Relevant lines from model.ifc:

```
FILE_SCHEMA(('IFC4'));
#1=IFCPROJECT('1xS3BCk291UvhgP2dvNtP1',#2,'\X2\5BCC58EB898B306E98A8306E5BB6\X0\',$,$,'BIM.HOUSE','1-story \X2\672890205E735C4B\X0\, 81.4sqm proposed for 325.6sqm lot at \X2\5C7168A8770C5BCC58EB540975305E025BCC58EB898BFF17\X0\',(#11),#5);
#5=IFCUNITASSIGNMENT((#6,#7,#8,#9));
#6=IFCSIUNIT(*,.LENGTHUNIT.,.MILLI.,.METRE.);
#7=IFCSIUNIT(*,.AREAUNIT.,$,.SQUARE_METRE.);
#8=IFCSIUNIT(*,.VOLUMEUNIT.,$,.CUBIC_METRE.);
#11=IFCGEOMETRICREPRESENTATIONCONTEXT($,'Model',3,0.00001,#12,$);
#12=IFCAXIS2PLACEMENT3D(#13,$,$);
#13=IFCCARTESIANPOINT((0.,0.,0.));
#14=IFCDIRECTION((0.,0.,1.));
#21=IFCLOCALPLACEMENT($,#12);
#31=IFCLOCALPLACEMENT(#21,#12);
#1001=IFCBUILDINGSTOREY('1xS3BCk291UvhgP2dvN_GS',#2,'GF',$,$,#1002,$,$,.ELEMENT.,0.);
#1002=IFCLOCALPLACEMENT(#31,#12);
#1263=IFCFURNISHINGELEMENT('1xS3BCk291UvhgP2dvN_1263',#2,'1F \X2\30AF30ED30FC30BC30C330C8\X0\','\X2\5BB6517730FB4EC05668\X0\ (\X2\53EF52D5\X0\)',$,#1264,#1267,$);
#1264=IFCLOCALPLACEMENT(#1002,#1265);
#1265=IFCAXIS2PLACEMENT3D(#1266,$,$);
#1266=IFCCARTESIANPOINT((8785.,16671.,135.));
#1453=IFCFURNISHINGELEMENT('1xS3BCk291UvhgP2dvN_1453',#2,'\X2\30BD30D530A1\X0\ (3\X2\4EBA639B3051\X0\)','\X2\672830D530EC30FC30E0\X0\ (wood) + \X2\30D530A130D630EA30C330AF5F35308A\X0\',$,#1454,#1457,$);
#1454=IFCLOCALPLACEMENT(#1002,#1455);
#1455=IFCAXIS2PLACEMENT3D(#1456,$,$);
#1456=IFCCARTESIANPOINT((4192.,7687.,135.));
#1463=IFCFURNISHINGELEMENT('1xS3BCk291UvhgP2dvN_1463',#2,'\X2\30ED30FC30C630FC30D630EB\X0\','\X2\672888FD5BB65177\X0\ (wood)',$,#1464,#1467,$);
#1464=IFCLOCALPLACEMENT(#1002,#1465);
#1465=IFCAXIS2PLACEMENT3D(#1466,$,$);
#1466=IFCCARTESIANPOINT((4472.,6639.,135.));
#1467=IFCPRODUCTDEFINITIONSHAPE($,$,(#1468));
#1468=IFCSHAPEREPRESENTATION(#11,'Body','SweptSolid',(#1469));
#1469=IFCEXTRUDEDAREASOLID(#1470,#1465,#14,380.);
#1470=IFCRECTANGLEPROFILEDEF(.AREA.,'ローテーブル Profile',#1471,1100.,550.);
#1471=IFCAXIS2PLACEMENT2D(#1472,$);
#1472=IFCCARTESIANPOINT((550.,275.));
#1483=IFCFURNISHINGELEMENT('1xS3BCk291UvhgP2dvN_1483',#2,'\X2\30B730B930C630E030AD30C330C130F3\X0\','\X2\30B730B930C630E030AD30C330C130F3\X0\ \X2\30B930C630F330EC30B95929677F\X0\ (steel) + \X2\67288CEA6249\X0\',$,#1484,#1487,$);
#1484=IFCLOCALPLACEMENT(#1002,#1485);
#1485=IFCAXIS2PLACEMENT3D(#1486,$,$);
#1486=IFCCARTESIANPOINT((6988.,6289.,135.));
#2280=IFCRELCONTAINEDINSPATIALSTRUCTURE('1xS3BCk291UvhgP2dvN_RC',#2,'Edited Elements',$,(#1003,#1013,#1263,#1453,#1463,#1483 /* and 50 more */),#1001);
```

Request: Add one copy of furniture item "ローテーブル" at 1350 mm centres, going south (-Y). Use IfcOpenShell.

```python
import numpy as np
import ifcopenshell
import ifcopenshell.api.geometry
import ifcopenshell.api.root
import ifcopenshell.util.element
import ifcopenshell.util.placement

model = ifcopenshell.open("model.ifc")


def reuse_history(source, copy):
    """copy_class also copies each property set's owner history, people and application; keep the originals."""
    for rel in copy.IsDefinedBy:
        if rel.is_a("IfcRelDefinesByProperties") and (history := rel.RelatingPropertyDefinition.OwnerHistory):
            rel.RelatingPropertyDefinition.OwnerHistory = source.OwnerHistory
            ifcopenshell.util.element.remove_deep2(model, history)


source = model.by_guid("1xS3BCk291UvhgP2dvN_1463")
base = ifcopenshell.util.placement.get_local_placement(source.ObjectPlacement)
step = np.array([0.0, -1.0, 0.0]) * 1350.0

for i in range(1, 2):
    copy = ifcopenshell.api.root.copy_class(model, product=source)
    copy.Representation = ifcopenshell.util.element.copy_deep(
        model, source.Representation, exclude=["IfcGeometricRepresentationContext", "IfcRepresentationMap"]
    )
    reuse_history(source, copy)
    matrix = base.copy()
    matrix[:3, 3] += i * step
    print("added at", matrix[:3, 3].round(3) + 0.0)
    ifcopenshell.api.geometry.edit_object_placement(model, product=copy, matrix=matrix, is_si=False)

model.write("model_rev.ifc")
```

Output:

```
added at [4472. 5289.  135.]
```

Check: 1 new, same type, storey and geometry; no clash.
